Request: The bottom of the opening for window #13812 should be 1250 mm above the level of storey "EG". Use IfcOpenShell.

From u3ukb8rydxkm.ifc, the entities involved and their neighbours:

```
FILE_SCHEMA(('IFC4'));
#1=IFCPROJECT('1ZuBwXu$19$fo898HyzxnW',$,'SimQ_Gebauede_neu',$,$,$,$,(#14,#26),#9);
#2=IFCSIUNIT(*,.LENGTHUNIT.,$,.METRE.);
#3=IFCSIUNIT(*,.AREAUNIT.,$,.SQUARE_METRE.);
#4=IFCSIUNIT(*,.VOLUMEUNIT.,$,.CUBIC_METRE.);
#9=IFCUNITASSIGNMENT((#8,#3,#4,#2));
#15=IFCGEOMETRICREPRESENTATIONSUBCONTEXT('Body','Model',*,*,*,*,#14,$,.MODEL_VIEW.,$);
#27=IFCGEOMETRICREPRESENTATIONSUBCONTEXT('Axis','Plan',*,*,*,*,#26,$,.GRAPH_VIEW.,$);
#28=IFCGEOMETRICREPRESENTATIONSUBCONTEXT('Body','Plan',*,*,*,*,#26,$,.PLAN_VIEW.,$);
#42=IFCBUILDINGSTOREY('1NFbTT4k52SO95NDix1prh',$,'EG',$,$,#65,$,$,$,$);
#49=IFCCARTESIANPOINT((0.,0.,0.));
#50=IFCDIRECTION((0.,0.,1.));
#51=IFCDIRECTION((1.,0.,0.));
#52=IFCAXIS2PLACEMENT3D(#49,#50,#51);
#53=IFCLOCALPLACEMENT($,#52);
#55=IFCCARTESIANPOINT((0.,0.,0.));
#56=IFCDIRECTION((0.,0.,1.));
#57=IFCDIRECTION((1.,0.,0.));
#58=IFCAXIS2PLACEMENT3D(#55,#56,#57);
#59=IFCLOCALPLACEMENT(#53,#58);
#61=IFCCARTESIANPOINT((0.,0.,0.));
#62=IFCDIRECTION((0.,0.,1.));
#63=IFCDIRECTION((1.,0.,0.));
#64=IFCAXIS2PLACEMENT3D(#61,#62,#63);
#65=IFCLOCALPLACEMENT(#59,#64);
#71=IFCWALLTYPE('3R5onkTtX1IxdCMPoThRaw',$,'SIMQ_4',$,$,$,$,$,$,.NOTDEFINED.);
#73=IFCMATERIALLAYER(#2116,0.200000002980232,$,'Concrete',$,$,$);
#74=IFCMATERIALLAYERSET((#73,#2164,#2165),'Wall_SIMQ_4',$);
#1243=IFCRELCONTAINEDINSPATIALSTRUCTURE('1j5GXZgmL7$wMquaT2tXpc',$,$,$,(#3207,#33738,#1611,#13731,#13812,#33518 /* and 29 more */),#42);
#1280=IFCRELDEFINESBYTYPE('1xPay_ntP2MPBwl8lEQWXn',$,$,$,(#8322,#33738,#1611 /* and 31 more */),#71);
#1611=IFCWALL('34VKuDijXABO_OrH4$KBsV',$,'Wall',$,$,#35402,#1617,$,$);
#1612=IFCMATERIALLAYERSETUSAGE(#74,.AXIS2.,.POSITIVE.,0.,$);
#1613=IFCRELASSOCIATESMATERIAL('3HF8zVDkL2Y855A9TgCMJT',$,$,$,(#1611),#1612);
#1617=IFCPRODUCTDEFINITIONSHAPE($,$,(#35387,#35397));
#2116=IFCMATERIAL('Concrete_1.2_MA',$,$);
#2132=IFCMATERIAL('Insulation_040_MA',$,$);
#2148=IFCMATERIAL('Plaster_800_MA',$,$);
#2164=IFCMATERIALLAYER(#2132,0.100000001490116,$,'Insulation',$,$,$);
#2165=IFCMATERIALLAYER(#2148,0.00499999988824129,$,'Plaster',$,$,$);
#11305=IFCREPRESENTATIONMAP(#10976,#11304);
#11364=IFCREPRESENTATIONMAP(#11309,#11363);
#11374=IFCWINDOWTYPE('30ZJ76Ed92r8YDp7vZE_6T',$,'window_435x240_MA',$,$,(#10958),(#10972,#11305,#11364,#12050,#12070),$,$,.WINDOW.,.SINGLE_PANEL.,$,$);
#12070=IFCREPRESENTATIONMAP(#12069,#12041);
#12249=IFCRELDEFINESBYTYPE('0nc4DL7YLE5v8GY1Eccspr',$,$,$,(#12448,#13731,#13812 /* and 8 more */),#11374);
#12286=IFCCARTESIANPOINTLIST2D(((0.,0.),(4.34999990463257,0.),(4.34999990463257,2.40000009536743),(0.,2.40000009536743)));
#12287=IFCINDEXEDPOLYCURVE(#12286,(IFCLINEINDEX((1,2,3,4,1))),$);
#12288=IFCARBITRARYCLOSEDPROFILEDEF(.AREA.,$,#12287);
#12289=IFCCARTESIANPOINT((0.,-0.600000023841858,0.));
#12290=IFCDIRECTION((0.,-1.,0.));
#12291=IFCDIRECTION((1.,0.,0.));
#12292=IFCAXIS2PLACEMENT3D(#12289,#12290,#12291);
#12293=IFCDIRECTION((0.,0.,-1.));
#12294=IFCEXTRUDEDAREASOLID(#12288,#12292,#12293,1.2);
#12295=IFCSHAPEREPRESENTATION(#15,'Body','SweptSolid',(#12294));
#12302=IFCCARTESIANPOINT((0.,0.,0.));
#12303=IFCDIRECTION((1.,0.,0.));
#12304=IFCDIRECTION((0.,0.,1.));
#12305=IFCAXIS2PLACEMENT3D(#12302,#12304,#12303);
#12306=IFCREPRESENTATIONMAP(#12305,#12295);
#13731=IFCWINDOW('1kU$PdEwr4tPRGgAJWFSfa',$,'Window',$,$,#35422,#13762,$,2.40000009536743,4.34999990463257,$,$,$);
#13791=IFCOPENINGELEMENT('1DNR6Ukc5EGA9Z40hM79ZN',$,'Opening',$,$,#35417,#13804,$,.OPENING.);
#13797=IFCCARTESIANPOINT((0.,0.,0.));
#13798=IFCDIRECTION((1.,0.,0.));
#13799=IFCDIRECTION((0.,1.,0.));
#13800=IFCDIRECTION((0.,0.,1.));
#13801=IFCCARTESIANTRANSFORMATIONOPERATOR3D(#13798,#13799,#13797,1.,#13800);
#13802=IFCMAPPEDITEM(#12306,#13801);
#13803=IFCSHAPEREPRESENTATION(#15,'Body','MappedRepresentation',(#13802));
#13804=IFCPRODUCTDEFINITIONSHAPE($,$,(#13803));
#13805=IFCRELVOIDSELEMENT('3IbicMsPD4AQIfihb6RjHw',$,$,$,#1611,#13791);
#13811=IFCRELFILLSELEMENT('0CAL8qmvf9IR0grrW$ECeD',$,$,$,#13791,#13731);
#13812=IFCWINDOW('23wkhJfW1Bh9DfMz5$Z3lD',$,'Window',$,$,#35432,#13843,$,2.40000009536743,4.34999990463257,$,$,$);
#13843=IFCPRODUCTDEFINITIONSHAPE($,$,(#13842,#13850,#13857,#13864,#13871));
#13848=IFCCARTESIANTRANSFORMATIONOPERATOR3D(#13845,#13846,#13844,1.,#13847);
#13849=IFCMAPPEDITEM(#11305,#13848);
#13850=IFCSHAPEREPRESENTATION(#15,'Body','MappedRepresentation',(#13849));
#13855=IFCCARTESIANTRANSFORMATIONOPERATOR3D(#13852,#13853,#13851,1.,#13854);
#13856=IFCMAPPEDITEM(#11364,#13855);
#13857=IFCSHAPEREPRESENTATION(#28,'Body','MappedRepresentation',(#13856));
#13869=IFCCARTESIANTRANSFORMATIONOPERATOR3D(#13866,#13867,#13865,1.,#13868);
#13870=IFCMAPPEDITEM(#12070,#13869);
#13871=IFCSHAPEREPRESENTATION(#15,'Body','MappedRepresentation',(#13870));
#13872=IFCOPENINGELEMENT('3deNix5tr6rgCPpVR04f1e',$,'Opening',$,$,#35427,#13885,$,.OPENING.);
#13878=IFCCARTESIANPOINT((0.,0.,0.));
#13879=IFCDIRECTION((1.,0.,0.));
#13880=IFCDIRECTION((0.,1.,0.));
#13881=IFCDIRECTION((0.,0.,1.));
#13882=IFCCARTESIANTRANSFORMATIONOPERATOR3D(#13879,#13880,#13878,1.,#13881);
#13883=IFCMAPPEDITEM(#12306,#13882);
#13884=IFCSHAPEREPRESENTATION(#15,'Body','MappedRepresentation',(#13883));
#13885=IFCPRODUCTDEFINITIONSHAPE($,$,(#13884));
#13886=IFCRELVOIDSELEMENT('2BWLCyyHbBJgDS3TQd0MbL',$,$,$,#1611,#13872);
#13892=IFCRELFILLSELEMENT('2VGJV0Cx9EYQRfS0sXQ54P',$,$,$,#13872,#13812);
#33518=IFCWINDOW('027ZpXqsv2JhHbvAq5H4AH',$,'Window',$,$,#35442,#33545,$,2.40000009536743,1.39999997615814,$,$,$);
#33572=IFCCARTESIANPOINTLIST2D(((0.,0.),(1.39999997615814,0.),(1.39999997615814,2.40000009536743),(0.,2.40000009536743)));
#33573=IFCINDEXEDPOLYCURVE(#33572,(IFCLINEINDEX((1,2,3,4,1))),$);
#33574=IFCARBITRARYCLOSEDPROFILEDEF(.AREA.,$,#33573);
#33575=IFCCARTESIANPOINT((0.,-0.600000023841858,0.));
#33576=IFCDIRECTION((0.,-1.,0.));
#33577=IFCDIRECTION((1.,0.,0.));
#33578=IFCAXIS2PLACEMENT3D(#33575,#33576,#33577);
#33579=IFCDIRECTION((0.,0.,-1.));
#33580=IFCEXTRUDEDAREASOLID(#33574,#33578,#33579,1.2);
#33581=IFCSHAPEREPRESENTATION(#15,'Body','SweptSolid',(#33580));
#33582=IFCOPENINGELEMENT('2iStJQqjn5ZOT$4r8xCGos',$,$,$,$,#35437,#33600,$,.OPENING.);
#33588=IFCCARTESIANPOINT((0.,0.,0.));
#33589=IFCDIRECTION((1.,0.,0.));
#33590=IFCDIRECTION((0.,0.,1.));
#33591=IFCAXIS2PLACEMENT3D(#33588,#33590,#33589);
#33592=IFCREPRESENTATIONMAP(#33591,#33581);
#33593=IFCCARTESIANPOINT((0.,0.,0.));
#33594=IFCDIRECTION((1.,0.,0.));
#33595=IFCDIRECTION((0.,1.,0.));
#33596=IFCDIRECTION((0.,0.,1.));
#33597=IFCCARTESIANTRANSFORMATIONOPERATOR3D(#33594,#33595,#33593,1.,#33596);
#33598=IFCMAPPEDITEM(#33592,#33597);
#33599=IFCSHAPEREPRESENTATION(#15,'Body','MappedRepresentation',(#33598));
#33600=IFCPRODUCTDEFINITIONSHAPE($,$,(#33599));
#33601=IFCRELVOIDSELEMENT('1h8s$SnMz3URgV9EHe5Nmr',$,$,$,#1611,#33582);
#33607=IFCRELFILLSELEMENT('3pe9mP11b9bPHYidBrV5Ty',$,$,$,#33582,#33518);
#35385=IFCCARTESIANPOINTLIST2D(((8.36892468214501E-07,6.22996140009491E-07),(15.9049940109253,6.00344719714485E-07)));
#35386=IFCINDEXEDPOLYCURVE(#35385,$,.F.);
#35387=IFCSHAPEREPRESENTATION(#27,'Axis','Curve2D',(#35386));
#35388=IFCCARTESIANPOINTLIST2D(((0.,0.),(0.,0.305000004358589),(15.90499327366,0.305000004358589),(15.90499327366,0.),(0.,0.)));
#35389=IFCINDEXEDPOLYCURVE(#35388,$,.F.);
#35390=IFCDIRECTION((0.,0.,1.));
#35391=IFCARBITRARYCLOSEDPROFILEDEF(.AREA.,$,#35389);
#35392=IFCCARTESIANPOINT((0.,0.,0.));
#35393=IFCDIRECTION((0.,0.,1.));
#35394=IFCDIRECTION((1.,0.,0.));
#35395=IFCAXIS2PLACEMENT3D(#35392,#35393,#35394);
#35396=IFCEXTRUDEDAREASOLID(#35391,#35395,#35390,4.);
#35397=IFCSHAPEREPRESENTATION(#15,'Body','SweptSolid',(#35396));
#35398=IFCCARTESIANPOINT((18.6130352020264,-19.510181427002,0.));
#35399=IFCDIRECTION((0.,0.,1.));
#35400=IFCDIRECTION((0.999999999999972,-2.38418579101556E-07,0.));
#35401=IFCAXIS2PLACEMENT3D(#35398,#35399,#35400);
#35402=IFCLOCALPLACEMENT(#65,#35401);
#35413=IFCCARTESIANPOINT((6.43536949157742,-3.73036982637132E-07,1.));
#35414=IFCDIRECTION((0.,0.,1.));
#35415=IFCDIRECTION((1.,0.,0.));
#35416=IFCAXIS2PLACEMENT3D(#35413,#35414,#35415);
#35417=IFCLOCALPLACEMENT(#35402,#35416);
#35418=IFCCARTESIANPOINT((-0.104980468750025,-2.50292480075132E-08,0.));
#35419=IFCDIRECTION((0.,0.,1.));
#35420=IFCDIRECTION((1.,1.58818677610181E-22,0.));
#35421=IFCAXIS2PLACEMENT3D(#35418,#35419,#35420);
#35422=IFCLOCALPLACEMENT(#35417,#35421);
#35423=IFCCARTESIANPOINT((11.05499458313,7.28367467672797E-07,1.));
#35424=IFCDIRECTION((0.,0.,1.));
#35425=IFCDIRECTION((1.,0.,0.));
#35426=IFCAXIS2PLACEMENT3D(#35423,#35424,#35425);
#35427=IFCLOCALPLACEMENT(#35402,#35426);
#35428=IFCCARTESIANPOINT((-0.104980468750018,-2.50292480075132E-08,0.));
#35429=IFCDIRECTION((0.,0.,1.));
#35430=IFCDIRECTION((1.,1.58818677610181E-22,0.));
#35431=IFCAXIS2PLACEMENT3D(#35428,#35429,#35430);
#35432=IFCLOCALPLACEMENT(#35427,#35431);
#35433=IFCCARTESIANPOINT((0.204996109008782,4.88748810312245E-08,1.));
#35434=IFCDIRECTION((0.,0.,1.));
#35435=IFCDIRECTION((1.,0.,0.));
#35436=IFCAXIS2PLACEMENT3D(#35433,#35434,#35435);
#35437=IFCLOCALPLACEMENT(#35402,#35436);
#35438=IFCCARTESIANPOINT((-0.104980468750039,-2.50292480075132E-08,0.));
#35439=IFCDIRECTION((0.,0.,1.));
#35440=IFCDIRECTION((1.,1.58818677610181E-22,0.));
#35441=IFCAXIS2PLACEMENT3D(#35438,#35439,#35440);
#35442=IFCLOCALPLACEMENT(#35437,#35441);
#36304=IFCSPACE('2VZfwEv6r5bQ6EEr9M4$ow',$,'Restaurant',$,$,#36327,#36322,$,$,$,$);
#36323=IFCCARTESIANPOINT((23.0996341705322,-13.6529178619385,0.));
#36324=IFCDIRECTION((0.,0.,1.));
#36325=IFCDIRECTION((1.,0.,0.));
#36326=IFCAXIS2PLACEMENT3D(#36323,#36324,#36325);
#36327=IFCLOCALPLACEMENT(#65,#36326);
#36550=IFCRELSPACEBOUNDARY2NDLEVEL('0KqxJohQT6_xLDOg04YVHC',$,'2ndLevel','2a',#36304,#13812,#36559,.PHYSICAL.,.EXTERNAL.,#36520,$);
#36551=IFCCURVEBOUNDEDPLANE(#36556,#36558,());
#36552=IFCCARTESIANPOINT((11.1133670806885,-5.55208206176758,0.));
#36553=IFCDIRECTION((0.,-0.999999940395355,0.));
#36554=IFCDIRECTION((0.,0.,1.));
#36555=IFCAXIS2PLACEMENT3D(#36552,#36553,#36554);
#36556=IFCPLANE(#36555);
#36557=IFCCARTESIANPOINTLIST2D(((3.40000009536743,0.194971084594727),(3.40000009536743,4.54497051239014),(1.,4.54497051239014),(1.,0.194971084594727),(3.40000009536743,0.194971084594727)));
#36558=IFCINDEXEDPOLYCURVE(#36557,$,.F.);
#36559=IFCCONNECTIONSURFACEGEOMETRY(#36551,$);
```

```python
import numpy as np
import ifcopenshell
import ifcopenshell.api.geometry
import ifcopenshell.geom
import ifcopenshell.util.element
import ifcopenshell.util.placement
import ifcopenshell.util.shape
import ifcopenshell.util.unit

model = ifcopenshell.open("u3ukb8rydxkm.ifc")
unit_scale = ifcopenshell.util.unit.calculate_unit_scale(model)

window = model.by_guid("23wkhJfW1Bh9DfMz5$Z3lD")
opening = window.FillsVoids[0].RelatingOpeningElement
storey = ifcopenshell.util.element.get_container(window, ifc_class="IfcBuildingStorey")
level = ifcopenshell.util.placement.get_local_placement(storey.ObjectPlacement)[2, 3]

# The opening's origin need not be at the sill, so measure its lowest point.
shape = ifcopenshell.geom.create_shape(ifcopenshell.geom.settings(), opening)
bottom = ifcopenshell.util.shape.get_shape_bottom_elevation(shape, shape.geometry) / unit_scale
dz = level + 1.25 / unit_scale - bottom

shift = np.array([0.0, 0.0, dz])
# The window is placed relative to its opening, so it follows when the opening moves.
matrix = ifcopenshell.util.placement.get_local_placement(opening.ObjectPlacement)
matrix[:3, 3] += shift
ifcopenshell.api.geometry.edit_object_placement(
    model, product=opening, matrix=matrix, is_si=False, should_transform_children=True
)

# Space boundary surfaces are stored in each space's coordinates; move them too.
for rel in window.ProvidesBoundaries:
    if not rel.ConnectionGeometry:
        continue
    surface = rel.ConnectionGeometry.SurfaceOnRelatingElement.BasisSurface
    space_matrix = ifcopenshell.util.placement.get_local_placement(rel.RelatingSpace.ObjectPlacement)
    point = np.array(surface.Position.Location.Coordinates) + space_matrix[:3, :3].T @ shift
    surface.Position = model.createIfcAxis2Placement3D(
        model.createIfcCartesianPoint(point.tolist()), surface.Position.Axis, surface.Position.RefDirection
    )

print(f"moved by {dz * unit_scale:+.3f} m")

model.write("u3ukb8rydxkm_v2.ifc")
```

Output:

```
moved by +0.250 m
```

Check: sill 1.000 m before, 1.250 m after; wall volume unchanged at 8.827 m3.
